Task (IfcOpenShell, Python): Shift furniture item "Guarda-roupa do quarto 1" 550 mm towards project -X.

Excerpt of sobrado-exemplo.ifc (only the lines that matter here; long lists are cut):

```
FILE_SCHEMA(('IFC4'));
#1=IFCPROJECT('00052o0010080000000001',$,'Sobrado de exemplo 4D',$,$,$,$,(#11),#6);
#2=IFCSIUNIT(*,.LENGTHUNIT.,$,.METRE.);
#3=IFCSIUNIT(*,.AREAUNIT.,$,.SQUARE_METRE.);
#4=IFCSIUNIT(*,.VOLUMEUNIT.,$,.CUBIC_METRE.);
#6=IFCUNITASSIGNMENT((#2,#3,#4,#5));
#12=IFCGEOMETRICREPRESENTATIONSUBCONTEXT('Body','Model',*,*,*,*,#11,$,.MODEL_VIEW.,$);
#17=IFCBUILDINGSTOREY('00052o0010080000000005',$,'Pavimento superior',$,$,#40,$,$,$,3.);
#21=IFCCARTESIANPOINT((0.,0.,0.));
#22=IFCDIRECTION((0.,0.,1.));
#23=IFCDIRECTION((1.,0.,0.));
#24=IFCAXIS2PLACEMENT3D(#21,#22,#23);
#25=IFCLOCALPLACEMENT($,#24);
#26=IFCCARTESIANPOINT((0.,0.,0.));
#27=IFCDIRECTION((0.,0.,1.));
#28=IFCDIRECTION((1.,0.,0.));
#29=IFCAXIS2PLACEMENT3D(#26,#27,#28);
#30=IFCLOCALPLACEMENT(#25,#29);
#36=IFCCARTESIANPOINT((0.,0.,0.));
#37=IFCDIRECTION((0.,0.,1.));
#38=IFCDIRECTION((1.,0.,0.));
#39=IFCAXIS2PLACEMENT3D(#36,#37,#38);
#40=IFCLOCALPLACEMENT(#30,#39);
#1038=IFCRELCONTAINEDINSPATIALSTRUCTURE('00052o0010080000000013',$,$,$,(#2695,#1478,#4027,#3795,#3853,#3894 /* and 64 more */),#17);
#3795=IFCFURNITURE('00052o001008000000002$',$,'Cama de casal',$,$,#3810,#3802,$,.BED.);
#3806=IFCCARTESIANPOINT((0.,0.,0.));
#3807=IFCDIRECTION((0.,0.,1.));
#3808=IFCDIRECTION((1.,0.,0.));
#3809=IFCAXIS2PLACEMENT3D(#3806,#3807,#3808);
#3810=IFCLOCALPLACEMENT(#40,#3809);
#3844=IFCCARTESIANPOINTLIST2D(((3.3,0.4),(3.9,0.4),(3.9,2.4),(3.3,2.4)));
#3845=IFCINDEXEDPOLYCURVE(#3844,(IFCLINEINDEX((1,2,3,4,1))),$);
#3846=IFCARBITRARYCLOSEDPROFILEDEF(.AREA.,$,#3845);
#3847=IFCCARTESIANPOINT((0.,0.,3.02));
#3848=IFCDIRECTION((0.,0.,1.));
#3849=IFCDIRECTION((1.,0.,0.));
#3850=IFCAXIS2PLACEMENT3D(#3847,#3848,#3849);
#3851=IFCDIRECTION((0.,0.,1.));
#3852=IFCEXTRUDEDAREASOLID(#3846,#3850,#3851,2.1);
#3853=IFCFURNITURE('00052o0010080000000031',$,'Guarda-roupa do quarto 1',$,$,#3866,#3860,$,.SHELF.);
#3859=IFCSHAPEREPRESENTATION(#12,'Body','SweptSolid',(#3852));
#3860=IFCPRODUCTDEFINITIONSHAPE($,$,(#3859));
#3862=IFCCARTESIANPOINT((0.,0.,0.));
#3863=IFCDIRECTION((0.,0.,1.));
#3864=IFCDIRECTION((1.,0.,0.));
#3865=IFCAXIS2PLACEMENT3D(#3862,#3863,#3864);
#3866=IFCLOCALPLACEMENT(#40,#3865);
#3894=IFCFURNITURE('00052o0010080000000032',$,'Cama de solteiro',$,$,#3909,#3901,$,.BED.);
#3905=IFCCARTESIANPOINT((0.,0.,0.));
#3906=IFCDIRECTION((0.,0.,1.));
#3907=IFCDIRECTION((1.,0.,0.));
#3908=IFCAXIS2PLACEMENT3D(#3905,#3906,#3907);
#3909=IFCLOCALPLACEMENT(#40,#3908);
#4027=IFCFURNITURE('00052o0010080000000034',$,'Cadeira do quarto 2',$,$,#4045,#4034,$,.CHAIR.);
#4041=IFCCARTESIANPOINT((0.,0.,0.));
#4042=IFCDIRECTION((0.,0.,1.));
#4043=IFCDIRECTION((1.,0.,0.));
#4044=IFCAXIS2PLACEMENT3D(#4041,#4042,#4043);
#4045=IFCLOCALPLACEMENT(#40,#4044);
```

```python
import ifcopenshell
import ifcopenshell.api.geometry
import ifcopenshell.util.placement

model = ifcopenshell.open("sobrado-exemplo.ifc")

item = model.by_guid("00052o0010080000000031")
matrix = ifcopenshell.util.placement.get_local_placement(item.ObjectPlacement)
matrix[0, 3] -= 0.55
ifcopenshell.api.geometry.edit_object_placement(model, product=item, matrix=matrix, is_si=False)

print(ifcopenshell.util.placement.get_local_placement(item.ObjectPlacement).round(3) + 0.0)

model.write("sobrado-exemplo_updated.ifc")
```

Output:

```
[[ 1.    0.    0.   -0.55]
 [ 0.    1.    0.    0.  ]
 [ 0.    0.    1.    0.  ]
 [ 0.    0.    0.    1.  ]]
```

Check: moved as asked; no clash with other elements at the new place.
